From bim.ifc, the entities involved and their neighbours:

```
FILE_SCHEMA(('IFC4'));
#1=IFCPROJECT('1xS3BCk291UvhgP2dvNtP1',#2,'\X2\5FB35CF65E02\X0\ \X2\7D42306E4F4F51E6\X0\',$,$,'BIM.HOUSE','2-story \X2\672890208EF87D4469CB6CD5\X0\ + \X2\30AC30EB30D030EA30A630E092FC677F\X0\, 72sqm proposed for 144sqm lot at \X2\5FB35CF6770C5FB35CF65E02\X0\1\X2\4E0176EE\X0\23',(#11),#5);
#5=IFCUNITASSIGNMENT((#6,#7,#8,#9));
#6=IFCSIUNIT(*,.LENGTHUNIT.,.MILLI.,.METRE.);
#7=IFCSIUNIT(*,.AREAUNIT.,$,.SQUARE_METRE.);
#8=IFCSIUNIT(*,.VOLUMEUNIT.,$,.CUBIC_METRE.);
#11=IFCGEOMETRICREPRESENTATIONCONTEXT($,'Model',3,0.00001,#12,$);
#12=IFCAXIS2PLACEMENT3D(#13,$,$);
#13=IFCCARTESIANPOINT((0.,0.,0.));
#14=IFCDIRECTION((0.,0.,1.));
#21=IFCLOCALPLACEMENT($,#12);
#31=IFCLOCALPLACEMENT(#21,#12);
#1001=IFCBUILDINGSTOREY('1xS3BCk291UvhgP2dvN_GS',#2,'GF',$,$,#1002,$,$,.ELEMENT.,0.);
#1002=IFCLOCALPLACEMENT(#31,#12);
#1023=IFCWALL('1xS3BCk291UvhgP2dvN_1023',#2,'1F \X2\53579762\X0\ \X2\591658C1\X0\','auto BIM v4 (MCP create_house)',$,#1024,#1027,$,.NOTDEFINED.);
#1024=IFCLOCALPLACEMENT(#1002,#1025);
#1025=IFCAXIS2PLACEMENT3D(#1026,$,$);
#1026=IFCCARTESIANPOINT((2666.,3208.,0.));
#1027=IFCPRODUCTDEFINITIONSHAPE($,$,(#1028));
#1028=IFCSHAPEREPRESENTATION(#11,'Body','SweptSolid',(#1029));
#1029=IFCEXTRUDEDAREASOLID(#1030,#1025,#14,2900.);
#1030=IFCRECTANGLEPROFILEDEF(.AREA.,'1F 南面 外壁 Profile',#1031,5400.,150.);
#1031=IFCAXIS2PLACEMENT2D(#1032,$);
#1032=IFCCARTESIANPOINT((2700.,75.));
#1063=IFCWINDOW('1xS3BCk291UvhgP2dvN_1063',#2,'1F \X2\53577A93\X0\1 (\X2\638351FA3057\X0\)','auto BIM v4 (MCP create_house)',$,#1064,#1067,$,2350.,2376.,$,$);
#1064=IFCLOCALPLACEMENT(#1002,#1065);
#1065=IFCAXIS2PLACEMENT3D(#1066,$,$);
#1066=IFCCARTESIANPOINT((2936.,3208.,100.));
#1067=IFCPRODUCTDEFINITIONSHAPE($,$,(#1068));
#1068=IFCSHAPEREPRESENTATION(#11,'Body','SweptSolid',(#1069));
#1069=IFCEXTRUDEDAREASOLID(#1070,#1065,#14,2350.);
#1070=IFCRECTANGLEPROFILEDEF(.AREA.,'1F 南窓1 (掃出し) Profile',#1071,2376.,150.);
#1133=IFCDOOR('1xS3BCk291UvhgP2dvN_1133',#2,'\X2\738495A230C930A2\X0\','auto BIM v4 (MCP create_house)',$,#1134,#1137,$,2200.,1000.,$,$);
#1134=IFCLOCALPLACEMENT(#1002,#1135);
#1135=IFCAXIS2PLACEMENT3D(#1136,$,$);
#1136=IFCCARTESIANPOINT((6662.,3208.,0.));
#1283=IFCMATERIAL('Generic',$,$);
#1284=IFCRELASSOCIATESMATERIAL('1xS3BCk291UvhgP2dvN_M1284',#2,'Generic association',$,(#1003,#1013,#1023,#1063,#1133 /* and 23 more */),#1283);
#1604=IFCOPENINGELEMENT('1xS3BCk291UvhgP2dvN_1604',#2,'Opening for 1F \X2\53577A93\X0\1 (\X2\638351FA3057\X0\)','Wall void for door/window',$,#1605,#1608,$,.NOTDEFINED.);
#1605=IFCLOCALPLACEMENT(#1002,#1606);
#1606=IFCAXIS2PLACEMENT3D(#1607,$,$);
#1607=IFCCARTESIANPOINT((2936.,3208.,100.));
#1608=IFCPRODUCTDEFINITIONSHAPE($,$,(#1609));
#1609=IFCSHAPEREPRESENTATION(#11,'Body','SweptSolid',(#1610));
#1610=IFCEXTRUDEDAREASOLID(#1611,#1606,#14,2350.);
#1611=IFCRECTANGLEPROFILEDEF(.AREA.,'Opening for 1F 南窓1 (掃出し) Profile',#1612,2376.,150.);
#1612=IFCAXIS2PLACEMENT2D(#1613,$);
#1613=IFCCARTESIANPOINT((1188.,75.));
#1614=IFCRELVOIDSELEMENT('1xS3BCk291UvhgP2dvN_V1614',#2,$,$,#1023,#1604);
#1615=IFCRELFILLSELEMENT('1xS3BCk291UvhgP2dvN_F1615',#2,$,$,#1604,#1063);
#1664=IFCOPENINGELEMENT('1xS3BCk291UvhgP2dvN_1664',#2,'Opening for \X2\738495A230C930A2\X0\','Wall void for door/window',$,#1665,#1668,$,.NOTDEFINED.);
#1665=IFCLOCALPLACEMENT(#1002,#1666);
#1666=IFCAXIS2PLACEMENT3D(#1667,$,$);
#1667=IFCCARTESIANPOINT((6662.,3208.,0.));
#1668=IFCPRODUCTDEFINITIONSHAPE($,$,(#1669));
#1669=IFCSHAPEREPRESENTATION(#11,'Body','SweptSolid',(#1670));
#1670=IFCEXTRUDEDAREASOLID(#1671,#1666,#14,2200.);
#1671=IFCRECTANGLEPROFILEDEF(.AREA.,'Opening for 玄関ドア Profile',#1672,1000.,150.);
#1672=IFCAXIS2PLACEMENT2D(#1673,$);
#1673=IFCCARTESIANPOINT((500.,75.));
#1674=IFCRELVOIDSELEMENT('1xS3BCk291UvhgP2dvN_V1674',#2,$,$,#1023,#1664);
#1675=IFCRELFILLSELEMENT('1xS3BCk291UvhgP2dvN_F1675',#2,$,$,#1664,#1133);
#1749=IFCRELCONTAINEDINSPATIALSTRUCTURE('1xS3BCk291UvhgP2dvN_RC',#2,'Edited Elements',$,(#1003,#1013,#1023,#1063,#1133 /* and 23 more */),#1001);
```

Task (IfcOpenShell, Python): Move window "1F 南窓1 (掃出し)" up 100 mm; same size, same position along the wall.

```python
import numpy as np
import ifcopenshell
import ifcopenshell.api.geometry
import ifcopenshell.util.placement
import ifcopenshell.util.unit

model = ifcopenshell.open("bim.ifc")
unit_scale = ifcopenshell.util.unit.calculate_unit_scale(model)

window = model.by_id(1063)
opening = window.FillsVoids[0].RelatingOpeningElement
dz = 100.0

shift = np.array([0.0, 0.0, dz])
# The window is not placed relative to its opening, so move both.
for product in (opening, window):
    matrix = ifcopenshell.util.placement.get_local_placement(product.ObjectPlacement)
    matrix[:3, 3] += shift
    ifcopenshell.api.geometry.edit_object_placement(model, product=product, matrix=matrix, is_si=False)

print(f"moved by {dz * unit_scale:+.3f} m")

model.write("bim_rev.ifc")
```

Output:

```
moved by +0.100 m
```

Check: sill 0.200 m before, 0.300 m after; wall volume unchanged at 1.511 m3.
